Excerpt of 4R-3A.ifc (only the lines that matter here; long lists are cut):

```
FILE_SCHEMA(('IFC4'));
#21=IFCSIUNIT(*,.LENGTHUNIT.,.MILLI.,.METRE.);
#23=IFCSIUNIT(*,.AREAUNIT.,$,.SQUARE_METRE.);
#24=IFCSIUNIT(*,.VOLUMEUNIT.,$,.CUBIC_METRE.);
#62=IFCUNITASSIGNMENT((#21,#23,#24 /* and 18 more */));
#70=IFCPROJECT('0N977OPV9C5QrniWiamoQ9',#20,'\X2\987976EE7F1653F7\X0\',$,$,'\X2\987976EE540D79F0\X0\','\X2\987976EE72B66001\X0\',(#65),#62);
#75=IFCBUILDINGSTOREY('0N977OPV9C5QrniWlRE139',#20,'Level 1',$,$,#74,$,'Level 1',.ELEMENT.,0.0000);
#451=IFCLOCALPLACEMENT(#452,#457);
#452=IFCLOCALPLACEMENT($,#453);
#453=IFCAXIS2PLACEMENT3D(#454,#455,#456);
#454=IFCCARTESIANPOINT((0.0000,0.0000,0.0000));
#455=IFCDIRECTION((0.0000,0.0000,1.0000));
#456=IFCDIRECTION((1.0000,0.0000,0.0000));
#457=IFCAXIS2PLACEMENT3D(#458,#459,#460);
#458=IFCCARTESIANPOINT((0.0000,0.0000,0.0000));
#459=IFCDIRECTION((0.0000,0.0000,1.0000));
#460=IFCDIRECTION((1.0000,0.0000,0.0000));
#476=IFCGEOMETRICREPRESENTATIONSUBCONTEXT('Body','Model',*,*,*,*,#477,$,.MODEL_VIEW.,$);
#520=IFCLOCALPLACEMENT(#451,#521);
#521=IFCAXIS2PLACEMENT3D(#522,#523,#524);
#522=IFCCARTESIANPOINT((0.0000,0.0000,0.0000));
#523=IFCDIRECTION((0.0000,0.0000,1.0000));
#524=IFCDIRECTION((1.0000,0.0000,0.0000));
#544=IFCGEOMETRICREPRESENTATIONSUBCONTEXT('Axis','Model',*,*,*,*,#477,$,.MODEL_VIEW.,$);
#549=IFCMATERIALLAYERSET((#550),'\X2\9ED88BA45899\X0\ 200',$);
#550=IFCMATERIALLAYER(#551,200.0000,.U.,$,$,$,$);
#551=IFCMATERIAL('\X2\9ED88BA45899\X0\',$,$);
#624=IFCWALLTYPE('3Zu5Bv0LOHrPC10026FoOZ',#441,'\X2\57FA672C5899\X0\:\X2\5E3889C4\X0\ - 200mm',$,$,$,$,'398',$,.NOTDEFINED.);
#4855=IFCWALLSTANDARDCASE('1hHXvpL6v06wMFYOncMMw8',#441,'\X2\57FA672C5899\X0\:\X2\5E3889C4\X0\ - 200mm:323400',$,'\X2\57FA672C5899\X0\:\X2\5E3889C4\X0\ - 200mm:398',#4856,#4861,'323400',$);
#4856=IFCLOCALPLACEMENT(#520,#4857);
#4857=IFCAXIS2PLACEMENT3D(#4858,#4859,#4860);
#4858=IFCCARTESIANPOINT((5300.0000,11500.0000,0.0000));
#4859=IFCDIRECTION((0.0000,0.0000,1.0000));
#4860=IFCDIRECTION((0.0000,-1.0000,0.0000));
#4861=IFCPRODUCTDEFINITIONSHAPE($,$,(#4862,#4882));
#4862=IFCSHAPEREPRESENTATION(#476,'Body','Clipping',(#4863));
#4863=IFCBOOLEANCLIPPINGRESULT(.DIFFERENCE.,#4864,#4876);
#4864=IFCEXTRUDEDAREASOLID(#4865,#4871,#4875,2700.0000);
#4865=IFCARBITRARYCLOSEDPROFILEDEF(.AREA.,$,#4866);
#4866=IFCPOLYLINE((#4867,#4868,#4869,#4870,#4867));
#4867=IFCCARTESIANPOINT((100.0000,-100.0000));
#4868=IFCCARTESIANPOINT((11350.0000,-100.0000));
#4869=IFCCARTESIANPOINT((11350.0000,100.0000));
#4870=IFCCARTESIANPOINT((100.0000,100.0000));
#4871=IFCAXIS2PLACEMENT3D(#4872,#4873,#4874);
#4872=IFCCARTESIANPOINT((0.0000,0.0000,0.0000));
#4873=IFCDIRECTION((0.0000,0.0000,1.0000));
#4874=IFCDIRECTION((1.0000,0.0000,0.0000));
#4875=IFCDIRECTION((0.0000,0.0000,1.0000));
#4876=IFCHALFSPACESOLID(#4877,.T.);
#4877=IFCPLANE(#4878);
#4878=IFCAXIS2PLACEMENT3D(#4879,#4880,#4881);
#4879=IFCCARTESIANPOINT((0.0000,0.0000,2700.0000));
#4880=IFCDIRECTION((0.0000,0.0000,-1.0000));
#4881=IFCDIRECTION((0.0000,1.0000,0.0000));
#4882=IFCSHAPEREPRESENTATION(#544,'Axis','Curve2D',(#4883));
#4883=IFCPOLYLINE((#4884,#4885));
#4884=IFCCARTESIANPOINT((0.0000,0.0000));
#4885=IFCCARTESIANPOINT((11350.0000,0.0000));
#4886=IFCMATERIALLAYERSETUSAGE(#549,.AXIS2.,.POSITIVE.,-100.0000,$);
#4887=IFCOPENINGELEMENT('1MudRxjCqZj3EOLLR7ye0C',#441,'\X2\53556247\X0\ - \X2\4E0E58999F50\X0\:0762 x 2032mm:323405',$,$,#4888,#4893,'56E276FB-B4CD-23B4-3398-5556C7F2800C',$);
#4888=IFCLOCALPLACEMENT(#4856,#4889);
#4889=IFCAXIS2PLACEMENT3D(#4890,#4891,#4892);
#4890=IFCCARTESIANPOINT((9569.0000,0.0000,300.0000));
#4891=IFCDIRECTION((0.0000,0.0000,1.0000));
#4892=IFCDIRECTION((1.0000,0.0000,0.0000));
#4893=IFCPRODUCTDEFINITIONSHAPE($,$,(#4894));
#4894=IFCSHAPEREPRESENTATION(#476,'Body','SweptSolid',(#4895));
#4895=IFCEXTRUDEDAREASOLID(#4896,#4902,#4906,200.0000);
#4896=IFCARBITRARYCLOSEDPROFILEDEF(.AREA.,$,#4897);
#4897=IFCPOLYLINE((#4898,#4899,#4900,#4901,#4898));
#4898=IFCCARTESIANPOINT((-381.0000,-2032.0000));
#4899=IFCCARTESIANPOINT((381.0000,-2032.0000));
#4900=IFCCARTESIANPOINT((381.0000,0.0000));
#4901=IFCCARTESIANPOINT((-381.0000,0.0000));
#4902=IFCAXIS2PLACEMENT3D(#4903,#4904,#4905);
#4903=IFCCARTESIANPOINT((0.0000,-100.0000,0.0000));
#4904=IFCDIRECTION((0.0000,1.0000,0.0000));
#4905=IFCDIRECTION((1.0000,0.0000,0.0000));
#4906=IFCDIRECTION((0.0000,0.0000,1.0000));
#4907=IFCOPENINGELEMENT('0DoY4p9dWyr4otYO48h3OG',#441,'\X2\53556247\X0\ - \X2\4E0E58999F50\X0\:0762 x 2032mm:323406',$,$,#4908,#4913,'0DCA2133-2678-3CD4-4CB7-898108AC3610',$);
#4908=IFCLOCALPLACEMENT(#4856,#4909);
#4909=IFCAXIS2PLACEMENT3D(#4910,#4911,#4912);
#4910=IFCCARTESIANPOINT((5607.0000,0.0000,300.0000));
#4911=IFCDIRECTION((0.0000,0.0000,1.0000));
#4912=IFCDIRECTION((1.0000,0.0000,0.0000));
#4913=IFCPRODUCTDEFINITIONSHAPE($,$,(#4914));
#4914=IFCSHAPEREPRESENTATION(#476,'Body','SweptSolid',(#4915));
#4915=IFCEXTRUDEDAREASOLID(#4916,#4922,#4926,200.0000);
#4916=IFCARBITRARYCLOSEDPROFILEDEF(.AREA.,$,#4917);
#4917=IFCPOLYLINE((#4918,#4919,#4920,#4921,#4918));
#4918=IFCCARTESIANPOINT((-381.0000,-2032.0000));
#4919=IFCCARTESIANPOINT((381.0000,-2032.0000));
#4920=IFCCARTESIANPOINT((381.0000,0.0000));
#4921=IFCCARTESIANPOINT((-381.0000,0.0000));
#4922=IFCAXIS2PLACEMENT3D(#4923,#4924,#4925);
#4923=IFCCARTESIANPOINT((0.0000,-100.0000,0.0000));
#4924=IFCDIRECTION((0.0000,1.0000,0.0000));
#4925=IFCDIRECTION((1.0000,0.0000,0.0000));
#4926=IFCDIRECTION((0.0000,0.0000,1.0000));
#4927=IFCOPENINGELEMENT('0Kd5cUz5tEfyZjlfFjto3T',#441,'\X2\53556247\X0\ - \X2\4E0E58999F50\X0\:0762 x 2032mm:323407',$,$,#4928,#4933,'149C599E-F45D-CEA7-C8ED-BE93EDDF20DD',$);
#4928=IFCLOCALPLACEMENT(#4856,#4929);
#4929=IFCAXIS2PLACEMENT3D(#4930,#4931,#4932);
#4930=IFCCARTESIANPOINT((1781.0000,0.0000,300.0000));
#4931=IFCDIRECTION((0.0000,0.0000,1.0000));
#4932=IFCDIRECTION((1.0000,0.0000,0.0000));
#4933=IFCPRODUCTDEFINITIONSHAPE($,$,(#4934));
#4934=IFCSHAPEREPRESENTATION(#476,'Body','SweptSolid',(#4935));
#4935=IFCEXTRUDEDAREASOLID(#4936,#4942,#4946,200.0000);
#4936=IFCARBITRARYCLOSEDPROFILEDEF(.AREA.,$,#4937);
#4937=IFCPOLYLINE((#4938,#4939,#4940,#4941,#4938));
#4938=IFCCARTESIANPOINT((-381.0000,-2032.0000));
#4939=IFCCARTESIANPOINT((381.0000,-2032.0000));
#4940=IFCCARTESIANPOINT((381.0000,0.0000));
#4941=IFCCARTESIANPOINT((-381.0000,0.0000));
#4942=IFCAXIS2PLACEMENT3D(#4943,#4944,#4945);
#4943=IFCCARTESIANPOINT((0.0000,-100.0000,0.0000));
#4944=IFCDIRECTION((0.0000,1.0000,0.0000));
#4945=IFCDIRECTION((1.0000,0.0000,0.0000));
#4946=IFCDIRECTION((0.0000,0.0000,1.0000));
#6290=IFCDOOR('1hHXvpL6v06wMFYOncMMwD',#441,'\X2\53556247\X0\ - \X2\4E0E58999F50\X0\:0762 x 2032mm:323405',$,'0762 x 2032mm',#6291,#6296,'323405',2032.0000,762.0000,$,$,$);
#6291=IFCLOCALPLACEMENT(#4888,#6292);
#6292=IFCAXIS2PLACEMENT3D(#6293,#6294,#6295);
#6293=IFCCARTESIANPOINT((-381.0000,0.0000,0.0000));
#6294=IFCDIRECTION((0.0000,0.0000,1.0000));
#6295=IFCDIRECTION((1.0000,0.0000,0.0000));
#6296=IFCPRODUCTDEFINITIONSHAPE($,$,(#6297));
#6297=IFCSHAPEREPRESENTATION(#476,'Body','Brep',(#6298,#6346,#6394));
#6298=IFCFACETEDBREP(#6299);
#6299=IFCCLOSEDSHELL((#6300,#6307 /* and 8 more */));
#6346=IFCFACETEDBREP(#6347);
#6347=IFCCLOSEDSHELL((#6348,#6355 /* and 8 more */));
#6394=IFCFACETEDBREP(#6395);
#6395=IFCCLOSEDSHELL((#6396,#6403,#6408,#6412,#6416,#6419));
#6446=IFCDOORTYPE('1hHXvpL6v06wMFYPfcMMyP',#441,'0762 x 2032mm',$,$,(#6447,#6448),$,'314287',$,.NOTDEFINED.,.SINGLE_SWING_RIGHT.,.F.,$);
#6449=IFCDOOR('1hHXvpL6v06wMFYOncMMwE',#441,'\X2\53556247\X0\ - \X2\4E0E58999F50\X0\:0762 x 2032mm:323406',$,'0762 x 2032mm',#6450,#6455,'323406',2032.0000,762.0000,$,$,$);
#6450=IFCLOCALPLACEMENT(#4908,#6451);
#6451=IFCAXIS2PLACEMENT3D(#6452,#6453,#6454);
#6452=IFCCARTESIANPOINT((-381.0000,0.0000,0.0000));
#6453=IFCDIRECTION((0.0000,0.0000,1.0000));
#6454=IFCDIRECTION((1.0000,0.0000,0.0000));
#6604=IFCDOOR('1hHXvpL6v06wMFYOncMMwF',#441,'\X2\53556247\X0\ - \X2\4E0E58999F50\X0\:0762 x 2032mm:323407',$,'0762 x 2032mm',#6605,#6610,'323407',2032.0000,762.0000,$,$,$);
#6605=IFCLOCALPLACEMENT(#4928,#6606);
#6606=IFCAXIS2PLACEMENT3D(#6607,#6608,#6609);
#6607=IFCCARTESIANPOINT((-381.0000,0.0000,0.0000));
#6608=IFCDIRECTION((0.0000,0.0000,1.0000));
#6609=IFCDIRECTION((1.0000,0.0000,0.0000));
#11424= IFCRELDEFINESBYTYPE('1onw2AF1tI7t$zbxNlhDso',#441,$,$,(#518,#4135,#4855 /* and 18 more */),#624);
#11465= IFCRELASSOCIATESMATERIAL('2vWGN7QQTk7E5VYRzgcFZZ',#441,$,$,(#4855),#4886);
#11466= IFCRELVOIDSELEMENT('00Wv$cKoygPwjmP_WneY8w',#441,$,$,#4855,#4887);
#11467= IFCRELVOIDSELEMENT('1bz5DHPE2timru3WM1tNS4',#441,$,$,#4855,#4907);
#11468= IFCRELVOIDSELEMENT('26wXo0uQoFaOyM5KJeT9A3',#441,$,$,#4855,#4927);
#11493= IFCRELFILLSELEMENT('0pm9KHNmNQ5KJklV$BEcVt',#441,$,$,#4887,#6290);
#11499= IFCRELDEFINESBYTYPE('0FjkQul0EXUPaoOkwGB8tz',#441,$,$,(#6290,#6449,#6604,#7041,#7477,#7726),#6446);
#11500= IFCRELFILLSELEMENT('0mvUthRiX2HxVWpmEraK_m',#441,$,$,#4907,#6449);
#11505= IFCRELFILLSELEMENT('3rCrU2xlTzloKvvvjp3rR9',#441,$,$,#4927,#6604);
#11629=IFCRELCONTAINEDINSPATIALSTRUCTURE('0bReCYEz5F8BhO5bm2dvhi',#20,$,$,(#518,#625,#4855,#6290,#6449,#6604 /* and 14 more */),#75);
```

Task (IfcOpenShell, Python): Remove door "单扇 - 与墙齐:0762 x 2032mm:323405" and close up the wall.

```python
import ifcopenshell
import ifcopenshell.api.feature
import ifcopenshell.api.root
import ifcopenshell.geom
import ifcopenshell.util.shape

model = ifcopenshell.open("4R-3A.ifc")
settings = ifcopenshell.geom.settings()


def volume(element):
    """Net volume in cubic metres, openings subtracted."""
    shape = ifcopenshell.geom.create_shape(settings, element)
    return ifcopenshell.util.shape.get_volume(shape.geometry)


door = model.by_guid("1hHXvpL6v06wMFYOncMMwD")
opening = door.FillsVoids[0].RelatingOpeningElement
wall = opening.VoidsElements[0].RelatingBuildingElement
before = volume(wall)

ifcopenshell.api.root.remove_product(model, product=door)
ifcopenshell.api.feature.remove_feature(model, feature=opening)

after = volume(wall)

print(f"wall volume {before:.3f} -> {after:.3f} m3")

model.write("4R-3A_edited.ifc")
```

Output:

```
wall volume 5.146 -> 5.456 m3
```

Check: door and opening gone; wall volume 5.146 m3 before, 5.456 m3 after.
